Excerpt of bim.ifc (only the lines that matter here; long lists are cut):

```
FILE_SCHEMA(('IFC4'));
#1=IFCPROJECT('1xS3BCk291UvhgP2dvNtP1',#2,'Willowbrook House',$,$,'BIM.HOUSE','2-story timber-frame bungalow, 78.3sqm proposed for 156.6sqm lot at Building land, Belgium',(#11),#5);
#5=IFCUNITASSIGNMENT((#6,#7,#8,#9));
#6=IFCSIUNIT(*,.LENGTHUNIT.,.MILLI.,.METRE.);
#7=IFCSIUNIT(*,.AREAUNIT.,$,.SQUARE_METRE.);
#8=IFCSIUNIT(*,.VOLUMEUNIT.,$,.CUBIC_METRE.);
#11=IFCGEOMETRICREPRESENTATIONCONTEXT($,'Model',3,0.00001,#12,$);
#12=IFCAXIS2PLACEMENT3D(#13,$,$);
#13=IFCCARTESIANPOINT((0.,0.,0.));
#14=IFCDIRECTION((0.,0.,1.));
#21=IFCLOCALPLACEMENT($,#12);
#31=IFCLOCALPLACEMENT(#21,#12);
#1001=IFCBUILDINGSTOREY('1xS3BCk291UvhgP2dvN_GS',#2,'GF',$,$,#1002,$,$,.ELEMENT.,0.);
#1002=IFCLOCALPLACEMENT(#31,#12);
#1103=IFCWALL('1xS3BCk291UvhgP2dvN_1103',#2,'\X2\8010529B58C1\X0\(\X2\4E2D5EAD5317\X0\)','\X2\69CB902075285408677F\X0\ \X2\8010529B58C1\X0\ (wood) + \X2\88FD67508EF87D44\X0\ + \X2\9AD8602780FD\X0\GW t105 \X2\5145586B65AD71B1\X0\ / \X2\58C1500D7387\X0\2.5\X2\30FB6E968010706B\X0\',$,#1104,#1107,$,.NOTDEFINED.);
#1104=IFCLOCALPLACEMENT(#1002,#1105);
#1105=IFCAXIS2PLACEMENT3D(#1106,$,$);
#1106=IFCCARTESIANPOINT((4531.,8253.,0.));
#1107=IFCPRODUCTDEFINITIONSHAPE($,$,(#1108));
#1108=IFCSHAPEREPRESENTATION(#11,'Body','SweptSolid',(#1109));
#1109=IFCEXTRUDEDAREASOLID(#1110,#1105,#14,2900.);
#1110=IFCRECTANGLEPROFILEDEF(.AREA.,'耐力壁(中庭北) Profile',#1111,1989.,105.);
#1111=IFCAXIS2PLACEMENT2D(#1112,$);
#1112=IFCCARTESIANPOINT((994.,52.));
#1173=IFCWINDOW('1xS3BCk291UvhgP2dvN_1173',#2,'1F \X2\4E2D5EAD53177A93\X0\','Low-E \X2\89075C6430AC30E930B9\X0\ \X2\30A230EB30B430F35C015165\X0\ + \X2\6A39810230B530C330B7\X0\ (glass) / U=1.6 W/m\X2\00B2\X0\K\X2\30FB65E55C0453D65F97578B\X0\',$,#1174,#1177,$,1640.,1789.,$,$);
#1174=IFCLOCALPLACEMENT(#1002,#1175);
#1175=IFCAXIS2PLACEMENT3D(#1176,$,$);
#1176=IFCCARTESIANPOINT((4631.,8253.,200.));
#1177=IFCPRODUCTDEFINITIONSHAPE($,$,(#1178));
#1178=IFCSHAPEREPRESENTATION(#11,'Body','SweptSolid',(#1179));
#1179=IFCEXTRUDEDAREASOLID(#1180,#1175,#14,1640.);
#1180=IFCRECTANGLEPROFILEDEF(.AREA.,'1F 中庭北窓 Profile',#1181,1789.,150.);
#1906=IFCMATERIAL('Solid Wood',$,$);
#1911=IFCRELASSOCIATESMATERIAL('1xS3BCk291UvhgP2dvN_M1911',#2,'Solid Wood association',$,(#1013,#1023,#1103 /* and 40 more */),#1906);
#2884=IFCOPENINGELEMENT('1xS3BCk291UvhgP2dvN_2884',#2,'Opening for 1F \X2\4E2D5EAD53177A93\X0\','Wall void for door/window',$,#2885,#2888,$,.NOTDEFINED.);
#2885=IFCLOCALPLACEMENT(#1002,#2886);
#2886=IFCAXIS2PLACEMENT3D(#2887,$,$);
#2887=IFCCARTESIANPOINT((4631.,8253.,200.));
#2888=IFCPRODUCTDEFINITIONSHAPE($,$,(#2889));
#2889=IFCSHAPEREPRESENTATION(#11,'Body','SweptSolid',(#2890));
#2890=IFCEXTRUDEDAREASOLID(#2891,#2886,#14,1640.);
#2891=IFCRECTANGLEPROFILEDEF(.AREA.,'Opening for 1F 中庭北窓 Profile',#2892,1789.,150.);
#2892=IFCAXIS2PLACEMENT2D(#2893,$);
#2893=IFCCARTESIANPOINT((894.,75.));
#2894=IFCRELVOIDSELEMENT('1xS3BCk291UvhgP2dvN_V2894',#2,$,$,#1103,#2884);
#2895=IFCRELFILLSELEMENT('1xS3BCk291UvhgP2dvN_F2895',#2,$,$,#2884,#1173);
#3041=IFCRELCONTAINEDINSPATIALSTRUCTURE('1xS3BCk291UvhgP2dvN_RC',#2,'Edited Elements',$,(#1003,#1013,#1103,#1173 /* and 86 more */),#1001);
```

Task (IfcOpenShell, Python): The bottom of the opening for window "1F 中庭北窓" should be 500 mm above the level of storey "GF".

```python
import numpy as np
import ifcopenshell
import ifcopenshell.api.geometry
import ifcopenshell.geom
import ifcopenshell.util.element
import ifcopenshell.util.placement
import ifcopenshell.util.shape
import ifcopenshell.util.unit

model = ifcopenshell.open("bim.ifc")
unit_scale = ifcopenshell.util.unit.calculate_unit_scale(model)

window = model.by_guid("1xS3BCk291UvhgP2dvN_1173")
opening = window.FillsVoids[0].RelatingOpeningElement
storey = ifcopenshell.util.element.get_container(window, ifc_class="IfcBuildingStorey")
level = ifcopenshell.util.placement.get_local_placement(storey.ObjectPlacement)[2, 3]

# The opening's origin need not be at the sill, so measure its lowest point.
shape = ifcopenshell.geom.create_shape(ifcopenshell.geom.settings(), opening)
bottom = ifcopenshell.util.shape.get_shape_bottom_elevation(shape, shape.geometry) / unit_scale
dz = level + 500.0 - bottom

shift = np.array([0.0, 0.0, dz])
# The window is not placed relative to its opening, so move both.
for product in (opening, window):
    matrix = ifcopenshell.util.placement.get_local_placement(product.ObjectPlacement)
    matrix[:3, 3] += shift
    ifcopenshell.api.geometry.edit_object_placement(model, product=product, matrix=matrix, is_si=False)

print(f"moved by {dz * unit_scale:+.3f} m")

model.write("bim_v2.ifc")
```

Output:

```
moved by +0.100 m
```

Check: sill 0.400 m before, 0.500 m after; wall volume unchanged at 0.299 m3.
